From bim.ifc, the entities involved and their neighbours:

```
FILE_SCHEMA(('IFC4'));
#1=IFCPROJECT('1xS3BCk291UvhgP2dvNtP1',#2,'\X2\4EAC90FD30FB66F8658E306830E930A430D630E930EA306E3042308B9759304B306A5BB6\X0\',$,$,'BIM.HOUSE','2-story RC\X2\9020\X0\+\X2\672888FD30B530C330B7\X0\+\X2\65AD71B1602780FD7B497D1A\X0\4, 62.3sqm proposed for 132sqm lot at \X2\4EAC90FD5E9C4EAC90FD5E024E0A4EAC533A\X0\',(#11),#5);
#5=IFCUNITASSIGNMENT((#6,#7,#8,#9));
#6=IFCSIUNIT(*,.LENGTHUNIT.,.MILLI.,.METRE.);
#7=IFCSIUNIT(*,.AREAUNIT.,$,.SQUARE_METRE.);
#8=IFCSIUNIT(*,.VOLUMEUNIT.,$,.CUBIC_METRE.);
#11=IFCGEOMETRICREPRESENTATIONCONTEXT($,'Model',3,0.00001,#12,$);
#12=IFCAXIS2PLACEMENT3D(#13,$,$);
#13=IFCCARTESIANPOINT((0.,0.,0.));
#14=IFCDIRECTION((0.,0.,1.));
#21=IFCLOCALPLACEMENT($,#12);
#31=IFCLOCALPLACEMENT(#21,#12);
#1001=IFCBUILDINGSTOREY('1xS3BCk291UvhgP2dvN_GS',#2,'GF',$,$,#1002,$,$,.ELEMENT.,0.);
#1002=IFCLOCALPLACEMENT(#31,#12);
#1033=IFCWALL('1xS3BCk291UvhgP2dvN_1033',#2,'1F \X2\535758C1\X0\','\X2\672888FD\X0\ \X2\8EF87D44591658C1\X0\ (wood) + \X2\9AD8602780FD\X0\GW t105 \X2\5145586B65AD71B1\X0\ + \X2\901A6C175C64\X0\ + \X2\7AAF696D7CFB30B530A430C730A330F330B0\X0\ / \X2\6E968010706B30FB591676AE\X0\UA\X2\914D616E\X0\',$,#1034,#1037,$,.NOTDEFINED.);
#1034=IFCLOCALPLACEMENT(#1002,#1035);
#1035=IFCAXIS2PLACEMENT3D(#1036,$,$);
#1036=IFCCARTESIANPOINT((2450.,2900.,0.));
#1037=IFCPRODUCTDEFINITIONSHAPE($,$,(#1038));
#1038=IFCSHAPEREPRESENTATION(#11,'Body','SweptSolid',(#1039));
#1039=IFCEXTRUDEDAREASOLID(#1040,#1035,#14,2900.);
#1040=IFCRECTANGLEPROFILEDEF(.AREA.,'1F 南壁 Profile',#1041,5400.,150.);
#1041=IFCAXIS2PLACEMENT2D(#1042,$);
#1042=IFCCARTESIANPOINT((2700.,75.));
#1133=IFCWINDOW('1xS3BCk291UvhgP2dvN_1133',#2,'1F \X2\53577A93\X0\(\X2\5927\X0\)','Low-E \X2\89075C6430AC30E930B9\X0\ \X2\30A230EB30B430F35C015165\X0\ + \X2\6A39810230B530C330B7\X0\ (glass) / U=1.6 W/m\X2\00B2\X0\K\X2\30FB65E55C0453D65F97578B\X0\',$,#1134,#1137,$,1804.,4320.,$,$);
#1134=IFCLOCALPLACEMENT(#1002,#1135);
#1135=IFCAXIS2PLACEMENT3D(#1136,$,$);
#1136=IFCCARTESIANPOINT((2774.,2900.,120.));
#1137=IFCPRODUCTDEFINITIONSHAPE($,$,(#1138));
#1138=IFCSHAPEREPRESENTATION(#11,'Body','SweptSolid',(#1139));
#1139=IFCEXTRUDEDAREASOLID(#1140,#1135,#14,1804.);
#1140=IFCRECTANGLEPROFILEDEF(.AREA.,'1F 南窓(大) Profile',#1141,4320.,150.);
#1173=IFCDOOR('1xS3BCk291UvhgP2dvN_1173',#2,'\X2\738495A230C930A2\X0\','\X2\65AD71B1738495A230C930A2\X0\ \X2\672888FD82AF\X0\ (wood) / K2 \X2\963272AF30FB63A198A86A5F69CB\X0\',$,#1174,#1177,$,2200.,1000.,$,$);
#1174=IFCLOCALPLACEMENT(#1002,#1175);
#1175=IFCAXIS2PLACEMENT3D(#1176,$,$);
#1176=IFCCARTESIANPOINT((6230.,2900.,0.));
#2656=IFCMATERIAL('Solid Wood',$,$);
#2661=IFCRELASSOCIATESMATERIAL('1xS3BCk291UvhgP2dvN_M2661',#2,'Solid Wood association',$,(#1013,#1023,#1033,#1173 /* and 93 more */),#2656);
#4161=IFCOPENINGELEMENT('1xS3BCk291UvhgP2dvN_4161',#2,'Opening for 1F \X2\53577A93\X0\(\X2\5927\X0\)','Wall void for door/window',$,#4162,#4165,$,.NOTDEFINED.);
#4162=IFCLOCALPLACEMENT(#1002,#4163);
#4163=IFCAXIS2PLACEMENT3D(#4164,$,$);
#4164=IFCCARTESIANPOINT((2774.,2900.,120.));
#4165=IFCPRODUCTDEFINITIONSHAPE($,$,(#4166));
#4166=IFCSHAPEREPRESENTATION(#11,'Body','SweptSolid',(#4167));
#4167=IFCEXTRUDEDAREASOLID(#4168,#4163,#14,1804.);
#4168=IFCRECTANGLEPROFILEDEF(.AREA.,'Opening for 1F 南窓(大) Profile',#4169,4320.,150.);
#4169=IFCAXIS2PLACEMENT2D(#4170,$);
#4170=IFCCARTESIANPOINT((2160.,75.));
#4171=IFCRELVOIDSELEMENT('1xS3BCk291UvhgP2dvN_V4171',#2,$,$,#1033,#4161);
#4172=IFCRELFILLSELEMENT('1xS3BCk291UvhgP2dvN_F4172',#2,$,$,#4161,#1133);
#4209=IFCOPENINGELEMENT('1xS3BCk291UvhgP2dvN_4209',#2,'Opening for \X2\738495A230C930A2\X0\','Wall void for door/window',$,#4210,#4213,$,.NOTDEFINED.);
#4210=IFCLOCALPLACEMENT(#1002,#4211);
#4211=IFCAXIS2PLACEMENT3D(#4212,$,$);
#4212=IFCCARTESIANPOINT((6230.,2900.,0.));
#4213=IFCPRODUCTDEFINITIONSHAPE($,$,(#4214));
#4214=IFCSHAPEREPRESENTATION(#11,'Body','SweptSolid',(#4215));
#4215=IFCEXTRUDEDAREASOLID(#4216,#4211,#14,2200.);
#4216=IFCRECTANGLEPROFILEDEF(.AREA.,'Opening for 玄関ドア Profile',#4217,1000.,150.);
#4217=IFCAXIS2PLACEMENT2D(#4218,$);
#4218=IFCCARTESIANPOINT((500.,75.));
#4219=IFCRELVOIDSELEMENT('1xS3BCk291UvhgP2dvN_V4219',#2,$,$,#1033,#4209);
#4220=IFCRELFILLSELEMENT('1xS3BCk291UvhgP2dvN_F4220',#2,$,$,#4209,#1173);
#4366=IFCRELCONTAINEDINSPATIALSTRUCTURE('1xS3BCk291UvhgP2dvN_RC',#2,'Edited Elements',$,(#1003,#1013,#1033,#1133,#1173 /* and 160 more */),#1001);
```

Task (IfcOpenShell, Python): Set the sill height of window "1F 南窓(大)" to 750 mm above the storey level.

```python
import numpy as np
import ifcopenshell
import ifcopenshell.api.geometry
import ifcopenshell.geom
import ifcopenshell.util.element
import ifcopenshell.util.placement
import ifcopenshell.util.shape
import ifcopenshell.util.unit

model = ifcopenshell.open("bim.ifc")
unit_scale = ifcopenshell.util.unit.calculate_unit_scale(model)

window = model.by_id(1133)
opening = window.FillsVoids[0].RelatingOpeningElement
storey = ifcopenshell.util.element.get_container(window, ifc_class="IfcBuildingStorey")
level = ifcopenshell.util.placement.get_local_placement(storey.ObjectPlacement)[2, 3]

# The opening's origin need not be at the sill, so measure its lowest point.
shape = ifcopenshell.geom.create_shape(ifcopenshell.geom.settings(), opening)
bottom = ifcopenshell.util.shape.get_shape_bottom_elevation(shape, shape.geometry) / unit_scale
dz = level + 0.75 / unit_scale - bottom

shift = np.array([0.0, 0.0, dz])
# The window is not placed relative to its opening, so move both.
for product in (opening, window):
    matrix = ifcopenshell.util.placement.get_local_placement(product.ObjectPlacement)
    matrix[:3, 3] += shift
    ifcopenshell.api.geometry.edit_object_placement(model, product=product, matrix=matrix, is_si=False)

print(f"moved by {dz * unit_scale:+.3f} m")

model.write("bim_edited.ifc")
```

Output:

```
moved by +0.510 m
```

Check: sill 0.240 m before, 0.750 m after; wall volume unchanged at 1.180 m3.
